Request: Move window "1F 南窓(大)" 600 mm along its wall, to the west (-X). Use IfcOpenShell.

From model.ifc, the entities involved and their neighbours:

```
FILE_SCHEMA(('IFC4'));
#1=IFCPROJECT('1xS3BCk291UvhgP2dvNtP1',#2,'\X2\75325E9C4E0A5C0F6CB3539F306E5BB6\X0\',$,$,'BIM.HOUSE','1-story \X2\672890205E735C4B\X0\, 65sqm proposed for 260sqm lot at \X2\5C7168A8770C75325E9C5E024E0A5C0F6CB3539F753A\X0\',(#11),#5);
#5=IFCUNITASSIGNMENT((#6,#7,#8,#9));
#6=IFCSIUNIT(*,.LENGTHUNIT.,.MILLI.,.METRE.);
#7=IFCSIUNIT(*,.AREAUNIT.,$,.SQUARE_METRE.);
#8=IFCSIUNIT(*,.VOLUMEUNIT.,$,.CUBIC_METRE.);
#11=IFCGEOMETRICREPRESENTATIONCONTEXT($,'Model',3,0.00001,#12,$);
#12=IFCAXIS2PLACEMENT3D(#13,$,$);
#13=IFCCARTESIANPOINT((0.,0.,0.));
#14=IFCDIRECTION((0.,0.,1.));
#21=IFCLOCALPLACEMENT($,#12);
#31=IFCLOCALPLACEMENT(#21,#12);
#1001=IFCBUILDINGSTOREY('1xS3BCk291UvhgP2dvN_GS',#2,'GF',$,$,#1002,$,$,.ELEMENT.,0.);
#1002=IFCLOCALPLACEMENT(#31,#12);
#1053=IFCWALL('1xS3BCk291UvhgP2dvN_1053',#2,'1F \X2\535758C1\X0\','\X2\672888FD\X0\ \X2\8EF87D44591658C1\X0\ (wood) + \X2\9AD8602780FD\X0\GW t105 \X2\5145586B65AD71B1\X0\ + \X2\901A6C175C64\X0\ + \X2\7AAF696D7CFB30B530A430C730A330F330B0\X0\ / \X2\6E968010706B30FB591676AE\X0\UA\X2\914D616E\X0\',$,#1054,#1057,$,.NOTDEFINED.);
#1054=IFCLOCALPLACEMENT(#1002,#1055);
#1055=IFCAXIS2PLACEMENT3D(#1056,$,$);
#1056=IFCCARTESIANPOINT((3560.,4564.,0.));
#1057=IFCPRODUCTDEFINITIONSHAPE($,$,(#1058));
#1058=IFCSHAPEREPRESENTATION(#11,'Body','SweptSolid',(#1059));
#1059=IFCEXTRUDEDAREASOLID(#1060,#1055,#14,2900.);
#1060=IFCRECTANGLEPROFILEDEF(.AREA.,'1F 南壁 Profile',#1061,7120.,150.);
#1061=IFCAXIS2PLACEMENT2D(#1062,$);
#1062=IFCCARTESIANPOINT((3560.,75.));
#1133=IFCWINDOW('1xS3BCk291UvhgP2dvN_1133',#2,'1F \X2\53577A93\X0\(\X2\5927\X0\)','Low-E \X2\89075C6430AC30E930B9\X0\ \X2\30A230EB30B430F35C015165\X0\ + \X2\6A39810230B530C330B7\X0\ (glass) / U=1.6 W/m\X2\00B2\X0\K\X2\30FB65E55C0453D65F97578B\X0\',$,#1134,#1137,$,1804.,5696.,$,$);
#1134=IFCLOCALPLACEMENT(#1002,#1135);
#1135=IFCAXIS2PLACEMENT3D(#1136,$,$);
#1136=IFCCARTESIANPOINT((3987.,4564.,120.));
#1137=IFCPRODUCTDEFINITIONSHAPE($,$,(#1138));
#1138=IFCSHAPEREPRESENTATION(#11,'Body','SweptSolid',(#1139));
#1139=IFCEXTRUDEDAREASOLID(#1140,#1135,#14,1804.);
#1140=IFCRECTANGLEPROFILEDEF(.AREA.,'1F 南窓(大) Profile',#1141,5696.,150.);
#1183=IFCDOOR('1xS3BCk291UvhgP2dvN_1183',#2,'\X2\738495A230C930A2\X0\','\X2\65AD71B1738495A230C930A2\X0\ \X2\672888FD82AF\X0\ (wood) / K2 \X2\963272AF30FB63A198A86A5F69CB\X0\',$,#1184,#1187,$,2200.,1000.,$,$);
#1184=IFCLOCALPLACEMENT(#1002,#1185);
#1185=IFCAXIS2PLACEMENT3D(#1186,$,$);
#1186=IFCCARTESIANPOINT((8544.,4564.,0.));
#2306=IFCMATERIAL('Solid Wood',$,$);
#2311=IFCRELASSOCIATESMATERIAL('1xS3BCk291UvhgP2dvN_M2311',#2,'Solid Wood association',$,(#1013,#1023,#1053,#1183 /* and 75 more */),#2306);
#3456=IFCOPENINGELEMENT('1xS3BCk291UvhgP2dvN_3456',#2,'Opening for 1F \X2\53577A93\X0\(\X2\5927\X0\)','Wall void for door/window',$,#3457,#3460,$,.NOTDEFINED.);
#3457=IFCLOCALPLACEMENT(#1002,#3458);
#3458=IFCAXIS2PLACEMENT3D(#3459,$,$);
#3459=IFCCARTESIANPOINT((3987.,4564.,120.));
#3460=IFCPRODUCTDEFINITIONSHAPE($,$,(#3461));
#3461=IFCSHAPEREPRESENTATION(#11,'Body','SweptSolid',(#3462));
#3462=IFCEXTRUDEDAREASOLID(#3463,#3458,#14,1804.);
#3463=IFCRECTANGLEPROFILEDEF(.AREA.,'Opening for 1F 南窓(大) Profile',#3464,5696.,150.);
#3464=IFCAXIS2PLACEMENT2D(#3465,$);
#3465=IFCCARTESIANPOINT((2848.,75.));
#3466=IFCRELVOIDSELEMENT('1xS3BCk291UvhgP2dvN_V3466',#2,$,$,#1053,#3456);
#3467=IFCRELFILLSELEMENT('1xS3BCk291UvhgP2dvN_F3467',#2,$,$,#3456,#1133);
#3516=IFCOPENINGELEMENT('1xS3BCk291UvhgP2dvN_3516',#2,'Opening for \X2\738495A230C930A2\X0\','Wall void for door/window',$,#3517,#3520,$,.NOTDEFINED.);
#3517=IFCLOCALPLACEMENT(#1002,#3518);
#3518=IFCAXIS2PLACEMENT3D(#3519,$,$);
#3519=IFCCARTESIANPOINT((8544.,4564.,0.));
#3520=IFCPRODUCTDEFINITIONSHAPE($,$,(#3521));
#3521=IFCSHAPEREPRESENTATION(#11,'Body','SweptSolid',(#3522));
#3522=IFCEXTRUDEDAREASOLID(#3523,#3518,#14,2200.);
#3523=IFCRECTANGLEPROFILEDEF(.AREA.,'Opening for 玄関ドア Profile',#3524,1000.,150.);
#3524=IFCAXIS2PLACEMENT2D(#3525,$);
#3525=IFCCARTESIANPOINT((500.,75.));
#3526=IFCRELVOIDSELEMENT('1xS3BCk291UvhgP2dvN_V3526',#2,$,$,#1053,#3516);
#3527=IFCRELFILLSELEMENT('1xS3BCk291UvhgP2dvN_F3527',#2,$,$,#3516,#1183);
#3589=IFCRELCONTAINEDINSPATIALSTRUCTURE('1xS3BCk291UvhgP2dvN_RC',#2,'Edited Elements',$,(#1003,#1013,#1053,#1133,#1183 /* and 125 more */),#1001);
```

```python
import ifcopenshell
import ifcopenshell.api.geometry
import ifcopenshell.util.placement

model = ifcopenshell.open("model.ifc")

window = model.by_id(1133)
opening = window.FillsVoids[0].RelatingOpeningElement
wall = opening.VoidsElements[0].RelatingBuildingElement

wall_matrix = ifcopenshell.util.placement.get_local_placement(wall.ObjectPlacement)
shift = wall_matrix[:3, 0] * -600.0
before = ifcopenshell.util.placement.get_local_placement(window.ObjectPlacement)[:3, 3].copy()

# The window is not placed relative to its opening, so move both.
for product in (opening, window):
    matrix = ifcopenshell.util.placement.get_local_placement(product.ObjectPlacement)
    matrix[:3, 3] += shift
    ifcopenshell.api.geometry.edit_object_placement(model, product=product, matrix=matrix, is_si=False)

after = ifcopenshell.util.placement.get_local_placement(window.ObjectPlacement)[:3, 3]
print("window moved by", (after - before).round(3) + 0.0)

model.write("model_rev.ifc")
```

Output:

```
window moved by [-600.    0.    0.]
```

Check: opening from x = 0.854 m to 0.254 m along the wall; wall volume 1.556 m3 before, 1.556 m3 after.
